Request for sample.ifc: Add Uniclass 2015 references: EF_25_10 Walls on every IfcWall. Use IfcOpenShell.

First a look at what the model holds.

```python
import ifcopenshell

model = ifcopenshell.open("sample.ifc")
print(model.schema)
print("classifications:", [c.Name for c in model.by_type("IfcClassification")])
for ifc_class in ("IfcDoor", "IfcRoof", "IfcStair", "IfcWall", "IfcWindow"):
    print(ifc_class, len(model.by_type(ifc_class)))
```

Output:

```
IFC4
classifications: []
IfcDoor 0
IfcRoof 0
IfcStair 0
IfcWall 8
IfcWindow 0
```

```python
import ifcopenshell
import ifcopenshell.api.classification

model = ifcopenshell.open("sample.ifc")

system = ifcopenshell.api.classification.add_classification(model, classification="Uniclass 2015")

codes = {
    "IfcWall": ("EF_25_10", "Walls"),
}
for ifc_class, (code, name) in codes.items():
    products = model.by_type(ifc_class)
    ifcopenshell.api.classification.add_reference(
        model, products=products, classification=system, identification=code, name=name
    )
    print(code, len(products))

model.write("sample_v2.ifc")
```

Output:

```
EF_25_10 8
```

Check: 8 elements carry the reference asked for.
